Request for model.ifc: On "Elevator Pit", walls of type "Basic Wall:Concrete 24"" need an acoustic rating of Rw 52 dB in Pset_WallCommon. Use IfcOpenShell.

First a look at what the model holds.

```python
import ifcopenshell
import ifcopenshell.util.element

model = ifcopenshell.open("model.ifc")
print(model.schema)
storey = next(s for s in model.by_type("IfcBuildingStorey") if s.Name == "Elevator Pit")
walls = [e for e in ifcopenshell.util.element.get_decomposition(storey) if e.is_a("IfcWall")]
seen = {}
for e in walls:
    element_type = ifcopenshell.util.element.get_type(e)
    key = (element_type.Name if element_type != e and element_type else None, ifcopenshell.util.element.get_pset(e, "Pset_WallCommon", "AcousticRating"))
    seen[key] = seen.get(key, 0) + 1
for (name, value), count in sorted(seen.items(), key=str):
    print(count, "x", name, "|", value)
```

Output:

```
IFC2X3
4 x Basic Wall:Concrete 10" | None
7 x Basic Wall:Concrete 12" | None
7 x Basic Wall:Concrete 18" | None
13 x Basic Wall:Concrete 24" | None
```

```python
import ifcopenshell
import ifcopenshell.api.pset
import ifcopenshell.util.element

model = ifcopenshell.open("model.ifc")

storey = next(s for s in model.by_type("IfcBuildingStorey") if s.Name == "Elevator Pit")
walls = [e for e in ifcopenshell.util.element.get_decomposition(storey) if e.is_a("IfcWall")]

count = 0
for e in walls:
    element_type = ifcopenshell.util.element.get_type(e)
    if element_type in (None, e) or element_type.Name != 'Basic Wall:Concrete 24"':
        continue
    # add_pset returns the element's existing set when there is one.
    pset = ifcopenshell.api.pset.add_pset(model, product=e, name="Pset_WallCommon")
    ifcopenshell.api.pset.edit_pset(model, pset=pset, properties={"AcousticRating": "Rw 52 dB"})
    count += 1

print(count, "walls updated")

model.write("model_v2.ifc")
```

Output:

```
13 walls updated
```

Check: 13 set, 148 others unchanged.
